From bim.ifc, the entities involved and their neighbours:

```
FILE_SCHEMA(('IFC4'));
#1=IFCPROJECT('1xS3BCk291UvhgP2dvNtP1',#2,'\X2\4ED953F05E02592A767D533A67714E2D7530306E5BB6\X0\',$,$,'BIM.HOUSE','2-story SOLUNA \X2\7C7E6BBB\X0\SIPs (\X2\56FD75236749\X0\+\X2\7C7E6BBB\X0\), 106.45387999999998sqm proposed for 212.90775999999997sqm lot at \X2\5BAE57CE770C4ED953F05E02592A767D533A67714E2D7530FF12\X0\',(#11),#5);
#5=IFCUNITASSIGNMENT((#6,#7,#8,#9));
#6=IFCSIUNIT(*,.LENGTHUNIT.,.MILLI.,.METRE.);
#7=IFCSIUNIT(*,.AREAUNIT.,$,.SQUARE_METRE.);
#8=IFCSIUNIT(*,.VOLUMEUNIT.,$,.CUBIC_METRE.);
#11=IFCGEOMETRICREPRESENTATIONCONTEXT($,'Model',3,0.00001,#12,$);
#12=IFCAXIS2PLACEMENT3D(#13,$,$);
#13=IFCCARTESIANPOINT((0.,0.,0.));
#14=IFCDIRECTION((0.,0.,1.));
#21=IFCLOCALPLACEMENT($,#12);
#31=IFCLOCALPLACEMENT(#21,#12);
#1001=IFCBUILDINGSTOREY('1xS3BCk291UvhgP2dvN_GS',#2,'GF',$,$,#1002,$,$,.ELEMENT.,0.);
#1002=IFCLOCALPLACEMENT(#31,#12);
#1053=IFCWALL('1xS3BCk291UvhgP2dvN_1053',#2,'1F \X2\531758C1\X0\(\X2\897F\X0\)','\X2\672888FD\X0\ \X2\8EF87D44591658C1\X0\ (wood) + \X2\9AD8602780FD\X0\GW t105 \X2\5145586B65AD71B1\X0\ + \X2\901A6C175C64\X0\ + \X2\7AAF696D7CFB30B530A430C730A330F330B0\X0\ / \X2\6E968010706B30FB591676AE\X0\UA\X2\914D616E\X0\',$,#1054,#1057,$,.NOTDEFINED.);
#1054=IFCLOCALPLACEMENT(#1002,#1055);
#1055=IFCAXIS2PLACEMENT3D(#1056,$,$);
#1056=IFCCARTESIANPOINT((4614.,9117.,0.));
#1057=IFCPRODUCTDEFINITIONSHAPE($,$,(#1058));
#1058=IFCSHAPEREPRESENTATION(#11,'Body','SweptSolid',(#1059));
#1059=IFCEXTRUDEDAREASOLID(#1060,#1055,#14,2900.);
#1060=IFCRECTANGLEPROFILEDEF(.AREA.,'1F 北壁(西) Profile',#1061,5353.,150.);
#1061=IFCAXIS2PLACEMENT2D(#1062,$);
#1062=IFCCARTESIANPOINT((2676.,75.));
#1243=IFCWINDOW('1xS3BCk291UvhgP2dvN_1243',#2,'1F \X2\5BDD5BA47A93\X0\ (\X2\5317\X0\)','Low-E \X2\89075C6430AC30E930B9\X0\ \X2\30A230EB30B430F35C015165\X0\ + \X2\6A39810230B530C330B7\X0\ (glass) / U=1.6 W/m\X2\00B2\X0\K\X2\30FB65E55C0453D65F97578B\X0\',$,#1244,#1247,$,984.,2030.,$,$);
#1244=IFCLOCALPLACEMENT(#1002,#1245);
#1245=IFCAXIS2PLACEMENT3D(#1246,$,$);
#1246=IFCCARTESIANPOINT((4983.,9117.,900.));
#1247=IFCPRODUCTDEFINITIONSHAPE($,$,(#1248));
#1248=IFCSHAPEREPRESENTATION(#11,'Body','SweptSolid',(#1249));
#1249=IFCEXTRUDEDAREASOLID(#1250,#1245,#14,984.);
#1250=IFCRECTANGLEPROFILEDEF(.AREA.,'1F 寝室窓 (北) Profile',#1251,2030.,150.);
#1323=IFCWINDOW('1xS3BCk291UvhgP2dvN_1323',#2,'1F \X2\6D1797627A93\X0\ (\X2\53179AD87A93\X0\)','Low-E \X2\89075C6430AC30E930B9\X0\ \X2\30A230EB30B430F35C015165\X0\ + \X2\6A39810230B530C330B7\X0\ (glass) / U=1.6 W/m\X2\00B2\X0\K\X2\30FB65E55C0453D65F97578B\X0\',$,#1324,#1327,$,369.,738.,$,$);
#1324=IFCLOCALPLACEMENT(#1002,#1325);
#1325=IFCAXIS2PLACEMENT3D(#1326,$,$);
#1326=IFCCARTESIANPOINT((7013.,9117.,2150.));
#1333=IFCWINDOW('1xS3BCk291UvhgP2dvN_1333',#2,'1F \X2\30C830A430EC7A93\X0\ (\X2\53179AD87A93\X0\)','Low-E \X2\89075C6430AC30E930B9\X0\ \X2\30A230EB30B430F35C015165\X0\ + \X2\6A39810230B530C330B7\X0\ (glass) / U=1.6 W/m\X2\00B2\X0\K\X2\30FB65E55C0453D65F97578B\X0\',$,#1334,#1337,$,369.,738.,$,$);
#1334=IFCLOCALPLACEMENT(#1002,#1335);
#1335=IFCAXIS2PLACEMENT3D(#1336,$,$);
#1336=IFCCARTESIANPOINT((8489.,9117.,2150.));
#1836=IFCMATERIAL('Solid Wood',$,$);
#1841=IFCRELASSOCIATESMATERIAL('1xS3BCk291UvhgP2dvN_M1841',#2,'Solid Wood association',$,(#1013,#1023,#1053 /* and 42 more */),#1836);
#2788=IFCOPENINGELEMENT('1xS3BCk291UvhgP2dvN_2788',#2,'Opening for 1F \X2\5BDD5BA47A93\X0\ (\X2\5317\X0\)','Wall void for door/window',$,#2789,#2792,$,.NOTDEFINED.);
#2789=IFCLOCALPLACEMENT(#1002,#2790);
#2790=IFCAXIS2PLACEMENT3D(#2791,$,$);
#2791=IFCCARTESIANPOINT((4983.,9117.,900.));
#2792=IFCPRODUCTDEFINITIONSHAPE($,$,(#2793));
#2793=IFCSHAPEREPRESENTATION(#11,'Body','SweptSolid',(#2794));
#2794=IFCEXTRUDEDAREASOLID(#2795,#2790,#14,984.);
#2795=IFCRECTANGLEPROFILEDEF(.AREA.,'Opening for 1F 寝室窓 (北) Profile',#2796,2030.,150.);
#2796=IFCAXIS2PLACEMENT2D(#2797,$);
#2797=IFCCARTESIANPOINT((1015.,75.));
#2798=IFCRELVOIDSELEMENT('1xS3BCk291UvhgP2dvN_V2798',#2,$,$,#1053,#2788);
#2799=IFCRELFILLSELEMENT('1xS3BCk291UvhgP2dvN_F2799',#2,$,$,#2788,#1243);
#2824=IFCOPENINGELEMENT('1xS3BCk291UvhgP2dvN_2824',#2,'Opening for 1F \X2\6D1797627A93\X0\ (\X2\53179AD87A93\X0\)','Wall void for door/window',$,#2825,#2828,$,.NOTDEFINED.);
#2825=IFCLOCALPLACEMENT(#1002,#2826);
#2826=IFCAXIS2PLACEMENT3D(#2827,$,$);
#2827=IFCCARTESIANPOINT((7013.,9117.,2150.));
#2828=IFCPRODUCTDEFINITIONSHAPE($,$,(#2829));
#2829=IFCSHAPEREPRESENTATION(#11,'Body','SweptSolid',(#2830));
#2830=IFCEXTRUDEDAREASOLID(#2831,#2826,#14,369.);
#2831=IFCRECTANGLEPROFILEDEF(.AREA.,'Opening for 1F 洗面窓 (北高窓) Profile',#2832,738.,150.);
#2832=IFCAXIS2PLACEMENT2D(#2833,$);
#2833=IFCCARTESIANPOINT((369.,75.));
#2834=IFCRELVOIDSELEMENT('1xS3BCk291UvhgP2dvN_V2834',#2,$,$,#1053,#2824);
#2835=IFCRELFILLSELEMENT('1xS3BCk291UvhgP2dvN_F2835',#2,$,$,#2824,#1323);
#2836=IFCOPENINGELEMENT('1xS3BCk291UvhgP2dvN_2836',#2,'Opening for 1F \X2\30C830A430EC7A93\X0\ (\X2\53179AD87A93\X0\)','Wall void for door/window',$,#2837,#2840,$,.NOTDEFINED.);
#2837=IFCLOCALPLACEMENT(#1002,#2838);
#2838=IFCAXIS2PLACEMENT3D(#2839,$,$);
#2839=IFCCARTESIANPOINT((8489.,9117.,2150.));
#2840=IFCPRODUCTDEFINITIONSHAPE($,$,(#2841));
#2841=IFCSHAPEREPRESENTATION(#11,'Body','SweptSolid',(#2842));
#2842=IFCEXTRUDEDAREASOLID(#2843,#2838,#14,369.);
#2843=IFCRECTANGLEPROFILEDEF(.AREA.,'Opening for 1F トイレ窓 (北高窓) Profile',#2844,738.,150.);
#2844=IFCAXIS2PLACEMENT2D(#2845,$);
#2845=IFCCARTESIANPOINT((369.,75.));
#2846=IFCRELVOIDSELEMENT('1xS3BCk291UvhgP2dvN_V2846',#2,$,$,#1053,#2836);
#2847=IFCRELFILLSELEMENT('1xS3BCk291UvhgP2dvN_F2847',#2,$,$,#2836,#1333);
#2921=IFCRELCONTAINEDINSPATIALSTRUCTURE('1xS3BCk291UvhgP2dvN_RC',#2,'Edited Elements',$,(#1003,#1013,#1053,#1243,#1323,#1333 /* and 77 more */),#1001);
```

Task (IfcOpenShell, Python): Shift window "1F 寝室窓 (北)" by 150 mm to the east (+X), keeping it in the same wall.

```python
import ifcopenshell
import ifcopenshell.api.geometry
import ifcopenshell.util.placement
import ifcopenshell.util.unit

model = ifcopenshell.open("bim.ifc")
unit_scale = ifcopenshell.util.unit.calculate_unit_scale(model)

window = model.by_guid("1xS3BCk291UvhgP2dvN_1243")
opening = window.FillsVoids[0].RelatingOpeningElement
wall = opening.VoidsElements[0].RelatingBuildingElement

wall_matrix = ifcopenshell.util.placement.get_local_placement(wall.ObjectPlacement)
shift = wall_matrix[:3, 0] * 0.15 / unit_scale
before = ifcopenshell.util.placement.get_local_placement(window.ObjectPlacement)[:3, 3].copy()

# The window is not placed relative to its opening, so move both.
for product in (opening, window):
    matrix = ifcopenshell.util.placement.get_local_placement(product.ObjectPlacement)
    matrix[:3, 3] += shift
    ifcopenshell.api.geometry.edit_object_placement(model, product=product, matrix=matrix, is_si=False)

after = ifcopenshell.util.placement.get_local_placement(window.ObjectPlacement)[:3, 3]
print("window moved by", (after - before).round(3) + 0.0)

model.write("bim_rev.ifc")
```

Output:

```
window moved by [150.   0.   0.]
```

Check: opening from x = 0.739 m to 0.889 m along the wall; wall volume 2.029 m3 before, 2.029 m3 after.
